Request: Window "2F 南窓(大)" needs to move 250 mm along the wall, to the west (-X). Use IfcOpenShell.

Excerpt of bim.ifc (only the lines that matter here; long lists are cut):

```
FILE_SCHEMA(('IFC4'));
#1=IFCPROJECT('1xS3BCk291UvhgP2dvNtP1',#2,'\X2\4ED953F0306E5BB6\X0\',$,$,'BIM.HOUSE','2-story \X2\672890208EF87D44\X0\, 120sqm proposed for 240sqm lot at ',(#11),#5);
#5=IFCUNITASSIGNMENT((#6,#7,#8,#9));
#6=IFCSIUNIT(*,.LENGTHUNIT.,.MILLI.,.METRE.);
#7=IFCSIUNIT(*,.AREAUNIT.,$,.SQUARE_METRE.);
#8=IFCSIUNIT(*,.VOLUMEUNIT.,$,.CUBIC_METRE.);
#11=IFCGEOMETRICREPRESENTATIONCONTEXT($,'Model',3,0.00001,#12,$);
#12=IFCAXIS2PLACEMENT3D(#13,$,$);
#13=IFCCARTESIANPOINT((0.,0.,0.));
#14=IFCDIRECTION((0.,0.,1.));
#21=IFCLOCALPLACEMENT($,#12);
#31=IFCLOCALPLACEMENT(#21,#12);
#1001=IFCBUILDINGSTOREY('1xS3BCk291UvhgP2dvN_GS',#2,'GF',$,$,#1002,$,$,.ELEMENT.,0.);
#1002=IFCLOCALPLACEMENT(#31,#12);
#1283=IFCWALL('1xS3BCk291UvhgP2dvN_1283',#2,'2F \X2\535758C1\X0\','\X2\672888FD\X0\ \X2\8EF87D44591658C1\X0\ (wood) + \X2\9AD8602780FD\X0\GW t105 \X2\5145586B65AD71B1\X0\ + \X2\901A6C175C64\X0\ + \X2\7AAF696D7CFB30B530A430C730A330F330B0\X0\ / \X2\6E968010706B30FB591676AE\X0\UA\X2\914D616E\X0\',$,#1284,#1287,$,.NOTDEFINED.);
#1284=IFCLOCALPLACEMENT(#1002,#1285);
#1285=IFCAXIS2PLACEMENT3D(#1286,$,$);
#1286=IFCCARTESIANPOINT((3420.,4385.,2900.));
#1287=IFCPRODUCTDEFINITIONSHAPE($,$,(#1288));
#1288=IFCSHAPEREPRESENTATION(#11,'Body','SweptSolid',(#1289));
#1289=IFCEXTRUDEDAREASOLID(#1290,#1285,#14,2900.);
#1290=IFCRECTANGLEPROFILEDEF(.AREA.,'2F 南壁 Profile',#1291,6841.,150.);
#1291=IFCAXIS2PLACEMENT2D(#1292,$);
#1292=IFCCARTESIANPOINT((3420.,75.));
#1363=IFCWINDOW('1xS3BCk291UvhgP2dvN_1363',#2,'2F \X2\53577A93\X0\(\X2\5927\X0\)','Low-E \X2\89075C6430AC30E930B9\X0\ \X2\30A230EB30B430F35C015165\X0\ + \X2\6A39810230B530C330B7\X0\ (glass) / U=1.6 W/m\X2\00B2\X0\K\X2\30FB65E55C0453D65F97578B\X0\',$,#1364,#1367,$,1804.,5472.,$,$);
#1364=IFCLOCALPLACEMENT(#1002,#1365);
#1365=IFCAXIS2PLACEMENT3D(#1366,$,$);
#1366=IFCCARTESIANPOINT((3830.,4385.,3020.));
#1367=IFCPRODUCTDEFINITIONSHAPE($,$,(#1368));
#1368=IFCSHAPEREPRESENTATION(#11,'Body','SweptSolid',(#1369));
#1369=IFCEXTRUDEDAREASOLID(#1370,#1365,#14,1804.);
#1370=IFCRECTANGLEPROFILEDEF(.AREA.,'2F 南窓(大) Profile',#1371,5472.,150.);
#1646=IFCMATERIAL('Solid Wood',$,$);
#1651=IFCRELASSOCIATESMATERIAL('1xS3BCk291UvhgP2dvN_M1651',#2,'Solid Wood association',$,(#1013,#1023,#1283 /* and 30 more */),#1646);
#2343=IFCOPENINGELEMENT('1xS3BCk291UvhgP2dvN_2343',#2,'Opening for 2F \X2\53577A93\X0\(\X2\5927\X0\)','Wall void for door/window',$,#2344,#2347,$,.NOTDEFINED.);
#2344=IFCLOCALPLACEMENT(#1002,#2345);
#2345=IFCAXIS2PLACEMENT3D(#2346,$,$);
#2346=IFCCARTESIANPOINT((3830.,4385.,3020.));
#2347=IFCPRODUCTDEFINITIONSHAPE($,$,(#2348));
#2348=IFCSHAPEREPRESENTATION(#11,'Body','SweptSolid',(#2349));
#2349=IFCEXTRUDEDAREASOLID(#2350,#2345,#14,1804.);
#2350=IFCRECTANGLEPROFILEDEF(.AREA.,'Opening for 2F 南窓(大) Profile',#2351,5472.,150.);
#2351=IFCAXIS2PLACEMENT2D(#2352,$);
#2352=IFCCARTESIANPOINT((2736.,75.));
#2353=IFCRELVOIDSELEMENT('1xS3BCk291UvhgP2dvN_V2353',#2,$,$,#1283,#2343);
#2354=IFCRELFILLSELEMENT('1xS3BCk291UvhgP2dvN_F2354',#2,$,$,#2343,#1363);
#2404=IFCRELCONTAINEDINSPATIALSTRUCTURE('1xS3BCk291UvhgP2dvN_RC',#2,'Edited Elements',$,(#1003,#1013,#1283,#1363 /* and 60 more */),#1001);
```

```python
import ifcopenshell
import ifcopenshell.api.geometry
import ifcopenshell.util.placement
import ifcopenshell.util.unit

model = ifcopenshell.open("bim.ifc")
unit_scale = ifcopenshell.util.unit.calculate_unit_scale(model)

window = model.by_guid("1xS3BCk291UvhgP2dvN_1363")
opening = window.FillsVoids[0].RelatingOpeningElement
wall = opening.VoidsElements[0].RelatingBuildingElement

wall_matrix = ifcopenshell.util.placement.get_local_placement(wall.ObjectPlacement)
shift = wall_matrix[:3, 0] * -0.25 / unit_scale
before = ifcopenshell.util.placement.get_local_placement(window.ObjectPlacement)[:3, 3].copy()

# The window is not placed relative to its opening, so move both.
for product in (opening, window):
    matrix = ifcopenshell.util.placement.get_local_placement(product.ObjectPlacement)
    matrix[:3, 3] += shift
    ifcopenshell.api.geometry.edit_object_placement(model, product=product, matrix=matrix, is_si=False)

after = ifcopenshell.util.placement.get_local_placement(window.ObjectPlacement)[:3, 3]
print("window moved by", (after - before).round(3) + 0.0)

model.write("bim-out.ifc")
```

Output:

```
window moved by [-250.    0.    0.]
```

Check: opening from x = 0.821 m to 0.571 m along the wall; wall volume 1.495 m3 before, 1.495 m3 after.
